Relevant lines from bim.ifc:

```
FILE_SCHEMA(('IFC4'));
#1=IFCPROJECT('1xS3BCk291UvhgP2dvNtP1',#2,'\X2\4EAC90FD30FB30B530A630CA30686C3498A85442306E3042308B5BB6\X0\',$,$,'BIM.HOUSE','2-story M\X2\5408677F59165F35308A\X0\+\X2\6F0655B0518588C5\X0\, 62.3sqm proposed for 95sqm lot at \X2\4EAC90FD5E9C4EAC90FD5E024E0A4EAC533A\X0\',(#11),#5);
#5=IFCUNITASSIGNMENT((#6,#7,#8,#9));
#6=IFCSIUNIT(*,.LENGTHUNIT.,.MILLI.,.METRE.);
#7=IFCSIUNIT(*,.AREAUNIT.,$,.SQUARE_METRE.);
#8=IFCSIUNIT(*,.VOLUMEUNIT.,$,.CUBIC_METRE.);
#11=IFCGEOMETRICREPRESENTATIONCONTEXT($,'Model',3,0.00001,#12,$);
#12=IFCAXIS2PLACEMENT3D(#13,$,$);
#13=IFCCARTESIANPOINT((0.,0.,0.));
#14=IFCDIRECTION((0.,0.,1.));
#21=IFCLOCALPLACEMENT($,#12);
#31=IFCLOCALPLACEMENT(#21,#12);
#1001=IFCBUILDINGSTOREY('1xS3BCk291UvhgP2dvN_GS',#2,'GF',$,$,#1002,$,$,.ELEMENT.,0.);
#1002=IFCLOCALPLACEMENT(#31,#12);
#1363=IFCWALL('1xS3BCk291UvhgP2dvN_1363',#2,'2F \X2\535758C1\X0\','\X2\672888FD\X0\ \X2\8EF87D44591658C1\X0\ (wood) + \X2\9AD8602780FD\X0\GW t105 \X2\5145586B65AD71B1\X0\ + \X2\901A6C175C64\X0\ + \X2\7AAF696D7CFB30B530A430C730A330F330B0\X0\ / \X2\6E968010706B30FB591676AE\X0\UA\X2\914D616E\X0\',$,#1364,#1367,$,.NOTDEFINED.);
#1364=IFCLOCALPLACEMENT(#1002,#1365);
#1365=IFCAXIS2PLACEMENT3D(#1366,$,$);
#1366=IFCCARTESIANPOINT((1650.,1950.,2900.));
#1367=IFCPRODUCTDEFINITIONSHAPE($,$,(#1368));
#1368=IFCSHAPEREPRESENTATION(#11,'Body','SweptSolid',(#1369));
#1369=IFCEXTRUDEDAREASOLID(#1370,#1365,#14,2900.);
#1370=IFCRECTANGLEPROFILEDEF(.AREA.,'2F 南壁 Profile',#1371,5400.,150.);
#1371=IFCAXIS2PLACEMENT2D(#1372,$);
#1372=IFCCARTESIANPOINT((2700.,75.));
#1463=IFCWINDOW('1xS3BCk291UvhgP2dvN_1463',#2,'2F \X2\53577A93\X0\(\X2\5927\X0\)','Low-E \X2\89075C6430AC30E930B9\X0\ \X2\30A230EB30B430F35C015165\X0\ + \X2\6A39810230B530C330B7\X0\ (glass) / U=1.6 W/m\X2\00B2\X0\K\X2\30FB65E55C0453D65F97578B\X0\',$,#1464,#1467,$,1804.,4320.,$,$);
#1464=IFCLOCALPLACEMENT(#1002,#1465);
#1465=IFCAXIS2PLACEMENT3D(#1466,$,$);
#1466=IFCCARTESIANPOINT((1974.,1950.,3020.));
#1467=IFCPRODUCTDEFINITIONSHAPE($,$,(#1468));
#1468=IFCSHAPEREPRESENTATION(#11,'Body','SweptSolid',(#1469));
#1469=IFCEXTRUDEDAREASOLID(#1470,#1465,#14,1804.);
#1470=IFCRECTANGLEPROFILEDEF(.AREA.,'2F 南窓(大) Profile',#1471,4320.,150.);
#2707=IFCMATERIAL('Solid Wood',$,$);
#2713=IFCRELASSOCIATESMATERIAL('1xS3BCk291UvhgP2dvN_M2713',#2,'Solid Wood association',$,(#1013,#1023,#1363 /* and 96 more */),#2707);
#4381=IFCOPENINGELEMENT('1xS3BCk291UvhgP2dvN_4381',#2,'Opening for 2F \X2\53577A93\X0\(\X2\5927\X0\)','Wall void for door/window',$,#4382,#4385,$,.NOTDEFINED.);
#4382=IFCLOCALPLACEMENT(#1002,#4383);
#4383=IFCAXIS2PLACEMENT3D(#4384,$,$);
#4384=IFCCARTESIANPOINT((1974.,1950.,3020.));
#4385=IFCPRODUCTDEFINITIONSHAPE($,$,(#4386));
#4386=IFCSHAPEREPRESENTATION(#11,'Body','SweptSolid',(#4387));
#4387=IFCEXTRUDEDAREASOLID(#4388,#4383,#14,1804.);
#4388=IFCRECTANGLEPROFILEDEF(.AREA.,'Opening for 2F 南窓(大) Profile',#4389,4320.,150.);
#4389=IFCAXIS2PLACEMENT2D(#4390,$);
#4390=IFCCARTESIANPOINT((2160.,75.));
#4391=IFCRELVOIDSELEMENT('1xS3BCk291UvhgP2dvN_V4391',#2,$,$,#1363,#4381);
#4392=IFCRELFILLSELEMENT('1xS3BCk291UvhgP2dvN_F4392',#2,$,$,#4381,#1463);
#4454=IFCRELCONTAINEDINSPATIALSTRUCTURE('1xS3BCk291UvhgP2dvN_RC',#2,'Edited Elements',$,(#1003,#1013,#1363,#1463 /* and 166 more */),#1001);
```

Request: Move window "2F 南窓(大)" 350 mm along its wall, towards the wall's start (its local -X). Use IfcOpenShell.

```python
import ifcopenshell
import ifcopenshell.api.geometry
import ifcopenshell.util.placement
import ifcopenshell.util.unit

model = ifcopenshell.open("bim.ifc")
unit_scale = ifcopenshell.util.unit.calculate_unit_scale(model)

window = model.by_guid("1xS3BCk291UvhgP2dvN_1463")
opening = window.FillsVoids[0].RelatingOpeningElement
wall = opening.VoidsElements[0].RelatingBuildingElement

wall_matrix = ifcopenshell.util.placement.get_local_placement(wall.ObjectPlacement)
shift = wall_matrix[:3, 0] * -0.35 / unit_scale
before = ifcopenshell.util.placement.get_local_placement(window.ObjectPlacement)[:3, 3].copy()

# The window is not placed relative to its opening, so move both.
for product in (opening, window):
    matrix = ifcopenshell.util.placement.get_local_placement(product.ObjectPlacement)
    matrix[:3, 3] += shift
    ifcopenshell.api.geometry.edit_object_placement(model, product=product, matrix=matrix, is_si=False)

after = ifcopenshell.util.placement.get_local_placement(window.ObjectPlacement)[:3, 3]
print("window moved by", (after - before).round(3) + 0.0)

model.write("bim-out.ifc")
```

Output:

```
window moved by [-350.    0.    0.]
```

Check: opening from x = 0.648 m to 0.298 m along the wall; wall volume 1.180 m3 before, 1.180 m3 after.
